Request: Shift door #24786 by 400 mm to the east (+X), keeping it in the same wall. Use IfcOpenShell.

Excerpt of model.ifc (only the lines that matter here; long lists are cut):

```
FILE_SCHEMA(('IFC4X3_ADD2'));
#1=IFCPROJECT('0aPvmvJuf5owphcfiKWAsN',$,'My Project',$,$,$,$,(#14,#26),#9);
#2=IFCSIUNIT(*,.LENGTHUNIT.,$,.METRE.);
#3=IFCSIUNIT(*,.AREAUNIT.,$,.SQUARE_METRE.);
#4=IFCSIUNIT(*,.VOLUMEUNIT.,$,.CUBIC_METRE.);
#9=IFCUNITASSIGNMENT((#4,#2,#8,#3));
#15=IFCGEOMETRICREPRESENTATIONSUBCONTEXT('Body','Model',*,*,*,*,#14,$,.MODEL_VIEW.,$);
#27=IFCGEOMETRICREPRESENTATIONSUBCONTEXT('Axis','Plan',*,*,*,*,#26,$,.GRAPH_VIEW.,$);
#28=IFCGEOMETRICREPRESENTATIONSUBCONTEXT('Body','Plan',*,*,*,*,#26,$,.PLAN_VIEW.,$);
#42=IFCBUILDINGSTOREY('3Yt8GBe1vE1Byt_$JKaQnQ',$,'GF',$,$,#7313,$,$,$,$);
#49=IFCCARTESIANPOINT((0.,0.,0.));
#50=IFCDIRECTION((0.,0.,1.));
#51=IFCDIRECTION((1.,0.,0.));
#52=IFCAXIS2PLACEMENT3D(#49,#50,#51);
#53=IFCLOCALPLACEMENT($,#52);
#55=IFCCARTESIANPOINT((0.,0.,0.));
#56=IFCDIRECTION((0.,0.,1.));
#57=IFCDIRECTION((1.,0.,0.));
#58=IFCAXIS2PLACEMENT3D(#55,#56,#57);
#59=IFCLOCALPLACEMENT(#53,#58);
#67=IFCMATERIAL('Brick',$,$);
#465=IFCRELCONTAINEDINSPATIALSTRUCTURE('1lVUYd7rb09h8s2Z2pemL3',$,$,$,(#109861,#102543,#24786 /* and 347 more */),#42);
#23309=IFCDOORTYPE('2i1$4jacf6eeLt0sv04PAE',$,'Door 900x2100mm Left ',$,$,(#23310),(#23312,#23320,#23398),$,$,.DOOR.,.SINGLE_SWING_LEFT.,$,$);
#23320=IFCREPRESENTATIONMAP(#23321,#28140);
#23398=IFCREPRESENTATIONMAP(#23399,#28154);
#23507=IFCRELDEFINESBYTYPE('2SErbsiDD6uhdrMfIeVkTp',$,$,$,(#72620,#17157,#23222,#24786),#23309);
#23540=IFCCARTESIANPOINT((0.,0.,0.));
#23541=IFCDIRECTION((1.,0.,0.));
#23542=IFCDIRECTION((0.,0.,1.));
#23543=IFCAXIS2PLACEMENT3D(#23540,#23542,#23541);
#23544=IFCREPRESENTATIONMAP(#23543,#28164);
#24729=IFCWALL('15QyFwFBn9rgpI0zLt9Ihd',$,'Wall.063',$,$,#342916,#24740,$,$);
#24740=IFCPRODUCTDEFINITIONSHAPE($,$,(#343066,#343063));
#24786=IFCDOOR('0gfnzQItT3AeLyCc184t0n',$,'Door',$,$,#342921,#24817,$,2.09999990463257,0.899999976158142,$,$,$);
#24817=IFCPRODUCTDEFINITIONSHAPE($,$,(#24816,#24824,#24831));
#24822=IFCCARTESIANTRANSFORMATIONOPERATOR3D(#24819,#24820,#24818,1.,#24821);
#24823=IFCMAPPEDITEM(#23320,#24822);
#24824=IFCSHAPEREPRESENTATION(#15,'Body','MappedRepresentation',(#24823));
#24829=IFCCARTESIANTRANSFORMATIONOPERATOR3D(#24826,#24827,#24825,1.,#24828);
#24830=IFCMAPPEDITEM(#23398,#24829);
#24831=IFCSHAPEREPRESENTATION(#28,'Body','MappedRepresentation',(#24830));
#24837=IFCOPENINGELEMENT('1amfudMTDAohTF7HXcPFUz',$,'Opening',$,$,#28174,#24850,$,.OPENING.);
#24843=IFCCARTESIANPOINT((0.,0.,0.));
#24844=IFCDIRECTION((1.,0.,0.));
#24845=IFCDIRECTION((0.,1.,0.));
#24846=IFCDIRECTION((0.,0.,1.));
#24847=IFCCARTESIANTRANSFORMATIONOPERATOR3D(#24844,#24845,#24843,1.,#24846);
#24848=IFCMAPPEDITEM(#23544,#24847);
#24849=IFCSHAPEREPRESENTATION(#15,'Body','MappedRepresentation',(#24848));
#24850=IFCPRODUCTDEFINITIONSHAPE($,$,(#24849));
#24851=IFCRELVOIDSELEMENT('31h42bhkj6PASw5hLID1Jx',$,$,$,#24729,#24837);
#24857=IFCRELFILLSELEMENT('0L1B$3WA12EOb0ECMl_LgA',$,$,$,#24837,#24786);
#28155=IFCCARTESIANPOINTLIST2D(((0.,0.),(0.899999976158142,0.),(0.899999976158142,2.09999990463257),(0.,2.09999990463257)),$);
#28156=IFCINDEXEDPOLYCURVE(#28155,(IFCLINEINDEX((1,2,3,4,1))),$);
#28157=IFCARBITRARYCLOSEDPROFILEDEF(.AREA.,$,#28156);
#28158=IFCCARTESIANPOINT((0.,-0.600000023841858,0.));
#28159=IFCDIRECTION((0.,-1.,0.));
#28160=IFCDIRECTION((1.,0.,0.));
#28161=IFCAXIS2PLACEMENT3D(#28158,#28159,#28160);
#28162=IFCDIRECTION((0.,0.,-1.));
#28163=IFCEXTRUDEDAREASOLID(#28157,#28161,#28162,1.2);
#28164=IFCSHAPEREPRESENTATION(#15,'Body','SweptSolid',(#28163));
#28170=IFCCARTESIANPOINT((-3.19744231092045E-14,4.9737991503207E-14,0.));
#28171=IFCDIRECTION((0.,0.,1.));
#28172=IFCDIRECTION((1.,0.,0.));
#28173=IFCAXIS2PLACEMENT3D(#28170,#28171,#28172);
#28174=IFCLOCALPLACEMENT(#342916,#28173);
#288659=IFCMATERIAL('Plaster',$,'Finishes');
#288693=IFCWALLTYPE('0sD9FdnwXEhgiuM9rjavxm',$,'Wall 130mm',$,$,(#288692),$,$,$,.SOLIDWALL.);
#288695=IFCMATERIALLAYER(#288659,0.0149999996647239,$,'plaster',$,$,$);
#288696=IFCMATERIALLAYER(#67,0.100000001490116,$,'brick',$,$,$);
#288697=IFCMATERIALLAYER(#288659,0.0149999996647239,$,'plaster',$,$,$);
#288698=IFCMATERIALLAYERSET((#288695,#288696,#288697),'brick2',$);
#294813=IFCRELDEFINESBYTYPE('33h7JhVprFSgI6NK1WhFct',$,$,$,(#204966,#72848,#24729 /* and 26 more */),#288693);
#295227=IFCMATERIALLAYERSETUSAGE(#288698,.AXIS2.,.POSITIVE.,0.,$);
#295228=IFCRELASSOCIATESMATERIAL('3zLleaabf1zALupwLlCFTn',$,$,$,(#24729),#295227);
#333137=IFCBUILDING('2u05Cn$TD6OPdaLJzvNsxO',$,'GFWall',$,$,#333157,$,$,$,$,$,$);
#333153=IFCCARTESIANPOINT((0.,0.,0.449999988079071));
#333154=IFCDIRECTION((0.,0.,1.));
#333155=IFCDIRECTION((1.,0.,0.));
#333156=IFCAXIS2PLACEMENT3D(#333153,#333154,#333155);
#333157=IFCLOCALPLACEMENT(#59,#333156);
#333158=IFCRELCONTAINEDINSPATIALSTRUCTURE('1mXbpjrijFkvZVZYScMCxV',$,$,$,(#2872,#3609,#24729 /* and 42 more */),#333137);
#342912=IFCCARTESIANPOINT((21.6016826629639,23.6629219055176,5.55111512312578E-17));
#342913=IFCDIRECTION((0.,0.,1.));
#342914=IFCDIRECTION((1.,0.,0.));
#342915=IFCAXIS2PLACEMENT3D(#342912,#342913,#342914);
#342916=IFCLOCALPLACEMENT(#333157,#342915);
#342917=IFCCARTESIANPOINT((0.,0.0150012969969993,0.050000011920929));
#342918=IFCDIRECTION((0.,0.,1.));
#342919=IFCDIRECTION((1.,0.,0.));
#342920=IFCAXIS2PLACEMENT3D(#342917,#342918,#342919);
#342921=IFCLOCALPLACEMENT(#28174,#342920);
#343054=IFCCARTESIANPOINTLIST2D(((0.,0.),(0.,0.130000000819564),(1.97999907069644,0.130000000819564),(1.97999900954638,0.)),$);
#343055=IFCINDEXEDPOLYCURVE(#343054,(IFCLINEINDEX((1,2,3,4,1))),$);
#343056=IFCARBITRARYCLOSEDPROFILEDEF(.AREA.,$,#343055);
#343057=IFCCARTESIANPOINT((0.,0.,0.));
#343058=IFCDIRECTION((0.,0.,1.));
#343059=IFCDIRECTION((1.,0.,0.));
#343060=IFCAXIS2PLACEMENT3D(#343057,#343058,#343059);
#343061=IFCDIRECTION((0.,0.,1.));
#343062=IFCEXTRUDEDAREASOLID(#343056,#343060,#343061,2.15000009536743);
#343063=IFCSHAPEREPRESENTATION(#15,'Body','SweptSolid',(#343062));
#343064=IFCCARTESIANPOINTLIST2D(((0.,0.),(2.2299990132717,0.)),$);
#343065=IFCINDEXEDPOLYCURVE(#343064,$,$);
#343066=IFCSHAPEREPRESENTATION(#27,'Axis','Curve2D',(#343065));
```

```python
import ifcopenshell
import ifcopenshell.api.geometry
import ifcopenshell.util.placement
import ifcopenshell.util.unit

model = ifcopenshell.open("model.ifc")
unit_scale = ifcopenshell.util.unit.calculate_unit_scale(model)

door = model.by_id(24786)
opening = door.FillsVoids[0].RelatingOpeningElement
wall = opening.VoidsElements[0].RelatingBuildingElement

wall_matrix = ifcopenshell.util.placement.get_local_placement(wall.ObjectPlacement)
shift = wall_matrix[:3, 0] * 0.4 / unit_scale
before = ifcopenshell.util.placement.get_local_placement(door.ObjectPlacement)[:3, 3].copy()

# The door is placed relative to its opening, so it follows when the opening moves.
matrix = ifcopenshell.util.placement.get_local_placement(opening.ObjectPlacement)
matrix[:3, 3] += shift
ifcopenshell.api.geometry.edit_object_placement(
    model, product=opening, matrix=matrix, is_si=False, should_transform_children=True
)

after = ifcopenshell.util.placement.get_local_placement(door.ObjectPlacement)[:3, 3]
print("door moved by", (after - before).round(3) + 0.0)

model.write("model_v2.ifc")
```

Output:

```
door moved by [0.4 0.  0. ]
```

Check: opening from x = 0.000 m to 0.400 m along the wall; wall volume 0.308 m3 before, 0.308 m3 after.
